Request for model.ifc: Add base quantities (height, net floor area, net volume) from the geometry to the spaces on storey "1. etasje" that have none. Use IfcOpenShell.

First a look at what the model holds.

```python
import ifcopenshell
import ifcopenshell.util.element
import ifcopenshell.util.unit

model = ifcopenshell.open("model.ifc")
print(model.schema)
for unit_type in ("LENGTHUNIT", "AREAUNIT", "VOLUMEUNIT"):
    print(unit_type, ifcopenshell.util.unit.calculate_unit_scale(model, unit_type))
storey = next(s for s in model.by_type("IfcBuildingStorey") if s.Name == "1. etasje")
spaces = [e for e in ifcopenshell.util.element.get_decomposition(storey) if e.is_a("IfcSpace")]
for e in sorted(spaces, key=lambda e: e.id()):
    print(e.id(), e.is_a(), e.Name, list(ifcopenshell.util.element.get_psets(e, qtos_only=True)), sep=" | ")
```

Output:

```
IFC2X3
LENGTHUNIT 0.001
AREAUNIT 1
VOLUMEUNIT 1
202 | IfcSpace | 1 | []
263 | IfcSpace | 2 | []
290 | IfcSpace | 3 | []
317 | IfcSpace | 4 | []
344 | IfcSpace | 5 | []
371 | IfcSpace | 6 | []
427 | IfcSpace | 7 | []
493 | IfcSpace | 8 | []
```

```python
import ifcopenshell
import ifcopenshell.api.pset
import ifcopenshell.geom
import ifcopenshell.util.element
import ifcopenshell.util.shape
import ifcopenshell.util.unit

model = ifcopenshell.open("model.ifc")
unit_scale = ifcopenshell.util.unit.calculate_unit_scale(model)
area_scale = ifcopenshell.util.unit.calculate_unit_scale(model, "AREAUNIT")
volume_scale = ifcopenshell.util.unit.calculate_unit_scale(model, "VOLUMEUNIT")
settings = ifcopenshell.geom.settings()

storey = next(s for s in model.by_type("IfcBuildingStorey") if s.Name == "1. etasje")
spaces = [e for e in ifcopenshell.util.element.get_decomposition(storey) if e.is_a("IfcSpace")]

for e in sorted(spaces, key=lambda e: e.id()):
    if ifcopenshell.util.element.get_psets(e, qtos_only=True, should_inherit=False):
        continue
    # Geometry comes back in metres, in the element's own axes.
    shape = ifcopenshell.geom.create_shape(settings, e)
    values = {
        "Height": ifcopenshell.util.shape.get_z(shape.geometry) / unit_scale,
        "NetFloorArea": ifcopenshell.util.shape.get_footprint_area(shape.geometry) / area_scale,
        "NetVolume": ifcopenshell.util.shape.get_volume(shape.geometry) / volume_scale,
    }
    qto = ifcopenshell.api.pset.add_qto(model, product=e, name="BaseQuantities")
    ifcopenshell.api.pset.edit_qto(model, qto=qto, properties=values)
    print(e.id(), {k: round(v, 3) for k, v in values.items()})

model.write("model_v2.ifc")
```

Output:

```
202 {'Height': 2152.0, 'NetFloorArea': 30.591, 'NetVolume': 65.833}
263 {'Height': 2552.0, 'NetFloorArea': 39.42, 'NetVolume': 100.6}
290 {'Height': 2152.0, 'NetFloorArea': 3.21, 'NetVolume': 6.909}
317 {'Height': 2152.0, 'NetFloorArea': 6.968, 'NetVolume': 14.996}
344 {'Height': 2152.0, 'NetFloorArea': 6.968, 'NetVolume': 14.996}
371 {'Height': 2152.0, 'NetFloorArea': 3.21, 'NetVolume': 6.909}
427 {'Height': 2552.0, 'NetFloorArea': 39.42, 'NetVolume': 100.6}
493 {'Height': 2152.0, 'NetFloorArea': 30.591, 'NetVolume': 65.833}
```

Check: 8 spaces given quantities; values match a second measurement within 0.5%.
